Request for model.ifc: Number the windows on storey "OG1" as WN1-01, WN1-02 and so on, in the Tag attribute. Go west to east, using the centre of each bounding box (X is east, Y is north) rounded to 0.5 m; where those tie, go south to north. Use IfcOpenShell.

First a look at what the model holds.

```python
import ifcopenshell
import ifcopenshell.util.element
import ifcopenshell.util.placement

model = ifcopenshell.open("model.ifc")
print(model.schema)
storey = next(s for s in model.by_type("IfcBuildingStorey") if s.Name == "OG1")
windows = [e for e in ifcopenshell.util.element.get_decomposition(storey) if e.is_a("IfcWindow")]
for e in sorted(windows, key=lambda e: e.id()):
    origin = ifcopenshell.util.placement.get_local_placement(e.ObjectPlacement)[:3, 3]
    print(e.id(), e.Tag, e.Name, origin.round(2) + 0.0, sep=" | ")
```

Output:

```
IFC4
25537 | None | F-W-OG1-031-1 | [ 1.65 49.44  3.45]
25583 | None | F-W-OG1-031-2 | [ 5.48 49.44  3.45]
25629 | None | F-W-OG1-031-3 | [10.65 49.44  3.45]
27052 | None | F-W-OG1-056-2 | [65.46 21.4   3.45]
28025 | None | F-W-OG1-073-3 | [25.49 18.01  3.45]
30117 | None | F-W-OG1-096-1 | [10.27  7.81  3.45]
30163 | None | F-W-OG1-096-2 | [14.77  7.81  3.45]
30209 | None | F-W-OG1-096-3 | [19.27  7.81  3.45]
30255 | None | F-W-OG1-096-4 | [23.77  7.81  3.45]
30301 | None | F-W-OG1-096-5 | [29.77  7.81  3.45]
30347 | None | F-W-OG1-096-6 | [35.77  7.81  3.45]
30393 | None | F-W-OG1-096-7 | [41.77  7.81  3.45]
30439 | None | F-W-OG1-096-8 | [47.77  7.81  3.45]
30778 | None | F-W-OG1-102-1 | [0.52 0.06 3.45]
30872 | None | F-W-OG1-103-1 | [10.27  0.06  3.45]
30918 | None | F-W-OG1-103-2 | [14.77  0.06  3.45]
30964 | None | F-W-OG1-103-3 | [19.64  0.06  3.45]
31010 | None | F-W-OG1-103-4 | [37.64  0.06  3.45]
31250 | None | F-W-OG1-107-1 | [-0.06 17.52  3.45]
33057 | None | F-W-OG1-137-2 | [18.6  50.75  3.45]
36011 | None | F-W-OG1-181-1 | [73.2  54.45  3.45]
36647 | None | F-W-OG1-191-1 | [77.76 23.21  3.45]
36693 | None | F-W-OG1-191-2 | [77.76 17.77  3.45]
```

```python
import ifcopenshell
import ifcopenshell.geom
import ifcopenshell.util.element
import ifcopenshell.util.shape

model = ifcopenshell.open("model.ifc")
settings = ifcopenshell.geom.settings()
settings.set("use-world-coords", True)


def centre(element):
    shape = ifcopenshell.geom.create_shape(settings, element)
    return ifcopenshell.util.shape.get_bbox_centroid(shape.geometry)


storey = next(s for s in model.by_type("IfcBuildingStorey") if s.Name == "OG1")
windows = [e for e in ifcopenshell.util.element.get_decomposition(storey) if e.is_a("IfcWindow")]

# Insertion points can sit at a corner or the storey origin, so sort by the geometry (in metres).
centres = {e: centre(e) for e in windows}
windows.sort(key=lambda e: (round(centres[e][0] / 0.5), centres[e][1]))

for i, e in enumerate(windows, start=1):
    number = f"WN1-{i:02d}"
    e.Tag = number
    print(e.id(), number)

model.write("model_edited.ifc")
```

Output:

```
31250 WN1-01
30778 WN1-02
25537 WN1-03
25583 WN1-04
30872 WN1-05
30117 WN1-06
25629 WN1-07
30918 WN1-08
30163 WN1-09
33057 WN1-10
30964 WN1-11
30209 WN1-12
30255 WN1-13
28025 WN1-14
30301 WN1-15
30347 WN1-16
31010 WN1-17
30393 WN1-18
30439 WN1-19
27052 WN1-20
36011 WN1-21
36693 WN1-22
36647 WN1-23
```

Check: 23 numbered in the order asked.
